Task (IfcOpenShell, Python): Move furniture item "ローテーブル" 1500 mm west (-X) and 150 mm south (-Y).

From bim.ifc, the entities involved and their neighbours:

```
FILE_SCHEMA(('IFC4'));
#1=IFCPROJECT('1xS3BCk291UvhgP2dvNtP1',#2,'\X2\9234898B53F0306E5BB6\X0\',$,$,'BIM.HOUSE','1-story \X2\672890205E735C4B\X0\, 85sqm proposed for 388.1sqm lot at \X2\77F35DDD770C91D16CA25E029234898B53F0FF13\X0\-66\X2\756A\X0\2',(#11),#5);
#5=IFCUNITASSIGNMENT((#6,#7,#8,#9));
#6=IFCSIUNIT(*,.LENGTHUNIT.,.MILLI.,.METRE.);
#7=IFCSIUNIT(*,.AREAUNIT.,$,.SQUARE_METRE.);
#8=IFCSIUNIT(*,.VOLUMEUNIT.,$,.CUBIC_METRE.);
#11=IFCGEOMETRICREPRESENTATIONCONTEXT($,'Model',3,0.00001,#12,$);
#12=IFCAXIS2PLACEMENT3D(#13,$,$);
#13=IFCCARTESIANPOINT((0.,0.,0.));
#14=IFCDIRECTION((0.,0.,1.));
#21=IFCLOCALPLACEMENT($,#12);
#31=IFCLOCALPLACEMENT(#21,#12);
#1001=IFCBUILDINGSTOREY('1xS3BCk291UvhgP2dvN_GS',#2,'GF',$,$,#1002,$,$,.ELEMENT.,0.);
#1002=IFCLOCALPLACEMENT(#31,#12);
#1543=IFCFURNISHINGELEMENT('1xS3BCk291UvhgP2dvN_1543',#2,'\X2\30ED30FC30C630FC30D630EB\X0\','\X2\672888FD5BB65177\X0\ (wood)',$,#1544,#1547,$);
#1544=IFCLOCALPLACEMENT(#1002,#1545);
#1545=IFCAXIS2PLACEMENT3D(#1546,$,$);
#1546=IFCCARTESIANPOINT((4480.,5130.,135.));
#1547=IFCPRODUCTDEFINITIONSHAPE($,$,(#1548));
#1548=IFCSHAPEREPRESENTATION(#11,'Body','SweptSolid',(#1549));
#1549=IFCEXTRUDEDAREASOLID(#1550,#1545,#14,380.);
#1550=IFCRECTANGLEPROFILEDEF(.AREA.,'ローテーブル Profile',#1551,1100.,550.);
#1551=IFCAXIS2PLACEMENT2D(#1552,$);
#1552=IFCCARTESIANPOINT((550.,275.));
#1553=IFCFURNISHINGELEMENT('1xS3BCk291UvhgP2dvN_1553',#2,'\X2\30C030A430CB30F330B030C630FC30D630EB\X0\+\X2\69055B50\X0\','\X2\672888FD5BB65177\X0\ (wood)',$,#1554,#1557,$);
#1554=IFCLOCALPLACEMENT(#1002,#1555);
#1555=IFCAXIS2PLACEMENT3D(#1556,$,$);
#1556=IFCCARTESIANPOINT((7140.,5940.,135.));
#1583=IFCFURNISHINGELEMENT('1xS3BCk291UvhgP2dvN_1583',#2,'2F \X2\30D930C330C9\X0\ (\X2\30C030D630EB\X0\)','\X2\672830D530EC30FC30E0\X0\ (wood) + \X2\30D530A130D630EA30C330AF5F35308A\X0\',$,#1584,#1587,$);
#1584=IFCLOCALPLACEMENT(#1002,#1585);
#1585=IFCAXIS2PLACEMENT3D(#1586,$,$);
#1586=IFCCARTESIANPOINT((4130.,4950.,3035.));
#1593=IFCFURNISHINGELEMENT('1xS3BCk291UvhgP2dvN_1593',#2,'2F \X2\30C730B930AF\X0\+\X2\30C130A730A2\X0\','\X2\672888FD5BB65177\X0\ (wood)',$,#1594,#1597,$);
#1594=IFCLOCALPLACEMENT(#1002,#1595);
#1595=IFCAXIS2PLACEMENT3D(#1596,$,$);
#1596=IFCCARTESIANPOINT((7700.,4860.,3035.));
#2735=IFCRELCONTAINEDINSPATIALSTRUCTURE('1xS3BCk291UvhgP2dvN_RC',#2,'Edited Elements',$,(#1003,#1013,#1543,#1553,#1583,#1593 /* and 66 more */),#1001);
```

```python
import ifcopenshell
import ifcopenshell.api.geometry
import ifcopenshell.util.placement

model = ifcopenshell.open("bim.ifc")

item = model.by_guid("1xS3BCk291UvhgP2dvN_1543")
matrix = ifcopenshell.util.placement.get_local_placement(item.ObjectPlacement)
matrix[0, 3] -= 1500.0
matrix[1, 3] -= 150.0
ifcopenshell.api.geometry.edit_object_placement(model, product=item, matrix=matrix, is_si=False)

print(ifcopenshell.util.placement.get_local_placement(item.ObjectPlacement).round(3) + 0.0)

model.write("bim_edited.ifc")
```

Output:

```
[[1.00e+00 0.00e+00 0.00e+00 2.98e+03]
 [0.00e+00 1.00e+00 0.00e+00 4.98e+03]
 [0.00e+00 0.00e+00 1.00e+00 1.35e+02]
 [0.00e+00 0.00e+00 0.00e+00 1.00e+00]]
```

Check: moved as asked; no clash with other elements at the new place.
